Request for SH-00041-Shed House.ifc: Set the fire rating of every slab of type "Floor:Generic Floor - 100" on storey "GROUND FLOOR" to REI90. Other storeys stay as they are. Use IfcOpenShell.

First a look at what the model holds.

```python
import ifcopenshell
import ifcopenshell.util.element

model = ifcopenshell.open("SH-00041-Shed House.ifc")
print(model.schema)
storey = next(s for s in model.by_type("IfcBuildingStorey") if s.Name == "GROUND FLOOR")
slabs = [e for e in ifcopenshell.util.element.get_decomposition(storey) if e.is_a("IfcSlab")]
seen = {}
for e in slabs:
    element_type = ifcopenshell.util.element.get_type(e)
    key = (element_type.Name if element_type != e and element_type else None, ifcopenshell.util.element.get_pset(e, "Pset_SlabCommon", "FireRating"))
    seen[key] = seen.get(key, 0) + 1
for (name, value), count in sorted(seen.items(), key=str):
    print(count, "x", name, "|", value)
```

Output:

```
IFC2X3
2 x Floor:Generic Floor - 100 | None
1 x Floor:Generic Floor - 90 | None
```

```python
import ifcopenshell
import ifcopenshell.api.pset
import ifcopenshell.util.element

model = ifcopenshell.open("SH-00041-Shed House.ifc")

storey = next(s for s in model.by_type("IfcBuildingStorey") if s.Name == "GROUND FLOOR")
slabs = [e for e in ifcopenshell.util.element.get_decomposition(storey) if e.is_a("IfcSlab")]

count = 0
for e in slabs:
    element_type = ifcopenshell.util.element.get_type(e)
    if element_type in (None, e) or element_type.Name != "Floor:Generic Floor - 100":
        continue
    # add_pset returns the element's existing set when there is one.
    pset = ifcopenshell.api.pset.add_pset(model, product=e, name="Pset_SlabCommon")
    ifcopenshell.api.pset.edit_pset(model, pset=pset, properties={"FireRating": "REI90"})
    count += 1

print(count, "slabs updated")

model.write("SH-00041-Shed House_rev.ifc")
```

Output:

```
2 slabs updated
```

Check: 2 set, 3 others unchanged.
